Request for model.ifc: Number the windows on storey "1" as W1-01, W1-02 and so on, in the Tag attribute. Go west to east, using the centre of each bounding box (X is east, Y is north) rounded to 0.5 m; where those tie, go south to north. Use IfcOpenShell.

First a look at what the model holds.

```python
import ifcopenshell
import ifcopenshell.util.element
import ifcopenshell.util.placement

model = ifcopenshell.open("model.ifc")
print(model.schema)
storey = next(s for s in model.by_type("IfcBuildingStorey") if s.Name == "1")
windows = [e for e in ifcopenshell.util.element.get_decomposition(storey) if e.is_a("IfcWindow")]
for e in sorted(windows, key=lambda e: e.id()):
    origin = ifcopenshell.util.placement.get_local_placement(e.ObjectPlacement)[:3, 3]
    print(e.id(), e.Tag, e.Name, origin.round(2) + 0.0, sep=" | ")
```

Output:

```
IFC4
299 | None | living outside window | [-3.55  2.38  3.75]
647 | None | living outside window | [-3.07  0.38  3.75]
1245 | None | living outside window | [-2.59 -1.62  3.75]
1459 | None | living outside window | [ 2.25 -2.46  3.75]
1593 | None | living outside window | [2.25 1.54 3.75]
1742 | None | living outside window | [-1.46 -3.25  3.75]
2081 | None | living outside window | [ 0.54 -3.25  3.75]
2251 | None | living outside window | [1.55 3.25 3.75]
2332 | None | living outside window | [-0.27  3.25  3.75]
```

```python
import ifcopenshell
import ifcopenshell.geom
import ifcopenshell.util.element
import ifcopenshell.util.shape

model = ifcopenshell.open("model.ifc")
settings = ifcopenshell.geom.settings()
settings.set("use-world-coords", True)


def centre(element):
    shape = ifcopenshell.geom.create_shape(settings, element)
    return ifcopenshell.util.shape.get_bbox_centroid(shape.geometry)


storey = next(s for s in model.by_type("IfcBuildingStorey") if s.Name == "1")
windows = [e for e in ifcopenshell.util.element.get_decomposition(storey) if e.is_a("IfcWindow")]

# Insertion points can sit at a corner or the storey origin, so sort by the geometry (in metres).
centres = {e: centre(e) for e in windows}
windows.sort(key=lambda e: (round(centres[e][0] / 0.5), centres[e][1]))

for i, e in enumerate(windows, start=1):
    number = f"W1-{i:02d}"
    e.Tag = number
    print(e.id(), number)

model.write("model_v2.ifc")
```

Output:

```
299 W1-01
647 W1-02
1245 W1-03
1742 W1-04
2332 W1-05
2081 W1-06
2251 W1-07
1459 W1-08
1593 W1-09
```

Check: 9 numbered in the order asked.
